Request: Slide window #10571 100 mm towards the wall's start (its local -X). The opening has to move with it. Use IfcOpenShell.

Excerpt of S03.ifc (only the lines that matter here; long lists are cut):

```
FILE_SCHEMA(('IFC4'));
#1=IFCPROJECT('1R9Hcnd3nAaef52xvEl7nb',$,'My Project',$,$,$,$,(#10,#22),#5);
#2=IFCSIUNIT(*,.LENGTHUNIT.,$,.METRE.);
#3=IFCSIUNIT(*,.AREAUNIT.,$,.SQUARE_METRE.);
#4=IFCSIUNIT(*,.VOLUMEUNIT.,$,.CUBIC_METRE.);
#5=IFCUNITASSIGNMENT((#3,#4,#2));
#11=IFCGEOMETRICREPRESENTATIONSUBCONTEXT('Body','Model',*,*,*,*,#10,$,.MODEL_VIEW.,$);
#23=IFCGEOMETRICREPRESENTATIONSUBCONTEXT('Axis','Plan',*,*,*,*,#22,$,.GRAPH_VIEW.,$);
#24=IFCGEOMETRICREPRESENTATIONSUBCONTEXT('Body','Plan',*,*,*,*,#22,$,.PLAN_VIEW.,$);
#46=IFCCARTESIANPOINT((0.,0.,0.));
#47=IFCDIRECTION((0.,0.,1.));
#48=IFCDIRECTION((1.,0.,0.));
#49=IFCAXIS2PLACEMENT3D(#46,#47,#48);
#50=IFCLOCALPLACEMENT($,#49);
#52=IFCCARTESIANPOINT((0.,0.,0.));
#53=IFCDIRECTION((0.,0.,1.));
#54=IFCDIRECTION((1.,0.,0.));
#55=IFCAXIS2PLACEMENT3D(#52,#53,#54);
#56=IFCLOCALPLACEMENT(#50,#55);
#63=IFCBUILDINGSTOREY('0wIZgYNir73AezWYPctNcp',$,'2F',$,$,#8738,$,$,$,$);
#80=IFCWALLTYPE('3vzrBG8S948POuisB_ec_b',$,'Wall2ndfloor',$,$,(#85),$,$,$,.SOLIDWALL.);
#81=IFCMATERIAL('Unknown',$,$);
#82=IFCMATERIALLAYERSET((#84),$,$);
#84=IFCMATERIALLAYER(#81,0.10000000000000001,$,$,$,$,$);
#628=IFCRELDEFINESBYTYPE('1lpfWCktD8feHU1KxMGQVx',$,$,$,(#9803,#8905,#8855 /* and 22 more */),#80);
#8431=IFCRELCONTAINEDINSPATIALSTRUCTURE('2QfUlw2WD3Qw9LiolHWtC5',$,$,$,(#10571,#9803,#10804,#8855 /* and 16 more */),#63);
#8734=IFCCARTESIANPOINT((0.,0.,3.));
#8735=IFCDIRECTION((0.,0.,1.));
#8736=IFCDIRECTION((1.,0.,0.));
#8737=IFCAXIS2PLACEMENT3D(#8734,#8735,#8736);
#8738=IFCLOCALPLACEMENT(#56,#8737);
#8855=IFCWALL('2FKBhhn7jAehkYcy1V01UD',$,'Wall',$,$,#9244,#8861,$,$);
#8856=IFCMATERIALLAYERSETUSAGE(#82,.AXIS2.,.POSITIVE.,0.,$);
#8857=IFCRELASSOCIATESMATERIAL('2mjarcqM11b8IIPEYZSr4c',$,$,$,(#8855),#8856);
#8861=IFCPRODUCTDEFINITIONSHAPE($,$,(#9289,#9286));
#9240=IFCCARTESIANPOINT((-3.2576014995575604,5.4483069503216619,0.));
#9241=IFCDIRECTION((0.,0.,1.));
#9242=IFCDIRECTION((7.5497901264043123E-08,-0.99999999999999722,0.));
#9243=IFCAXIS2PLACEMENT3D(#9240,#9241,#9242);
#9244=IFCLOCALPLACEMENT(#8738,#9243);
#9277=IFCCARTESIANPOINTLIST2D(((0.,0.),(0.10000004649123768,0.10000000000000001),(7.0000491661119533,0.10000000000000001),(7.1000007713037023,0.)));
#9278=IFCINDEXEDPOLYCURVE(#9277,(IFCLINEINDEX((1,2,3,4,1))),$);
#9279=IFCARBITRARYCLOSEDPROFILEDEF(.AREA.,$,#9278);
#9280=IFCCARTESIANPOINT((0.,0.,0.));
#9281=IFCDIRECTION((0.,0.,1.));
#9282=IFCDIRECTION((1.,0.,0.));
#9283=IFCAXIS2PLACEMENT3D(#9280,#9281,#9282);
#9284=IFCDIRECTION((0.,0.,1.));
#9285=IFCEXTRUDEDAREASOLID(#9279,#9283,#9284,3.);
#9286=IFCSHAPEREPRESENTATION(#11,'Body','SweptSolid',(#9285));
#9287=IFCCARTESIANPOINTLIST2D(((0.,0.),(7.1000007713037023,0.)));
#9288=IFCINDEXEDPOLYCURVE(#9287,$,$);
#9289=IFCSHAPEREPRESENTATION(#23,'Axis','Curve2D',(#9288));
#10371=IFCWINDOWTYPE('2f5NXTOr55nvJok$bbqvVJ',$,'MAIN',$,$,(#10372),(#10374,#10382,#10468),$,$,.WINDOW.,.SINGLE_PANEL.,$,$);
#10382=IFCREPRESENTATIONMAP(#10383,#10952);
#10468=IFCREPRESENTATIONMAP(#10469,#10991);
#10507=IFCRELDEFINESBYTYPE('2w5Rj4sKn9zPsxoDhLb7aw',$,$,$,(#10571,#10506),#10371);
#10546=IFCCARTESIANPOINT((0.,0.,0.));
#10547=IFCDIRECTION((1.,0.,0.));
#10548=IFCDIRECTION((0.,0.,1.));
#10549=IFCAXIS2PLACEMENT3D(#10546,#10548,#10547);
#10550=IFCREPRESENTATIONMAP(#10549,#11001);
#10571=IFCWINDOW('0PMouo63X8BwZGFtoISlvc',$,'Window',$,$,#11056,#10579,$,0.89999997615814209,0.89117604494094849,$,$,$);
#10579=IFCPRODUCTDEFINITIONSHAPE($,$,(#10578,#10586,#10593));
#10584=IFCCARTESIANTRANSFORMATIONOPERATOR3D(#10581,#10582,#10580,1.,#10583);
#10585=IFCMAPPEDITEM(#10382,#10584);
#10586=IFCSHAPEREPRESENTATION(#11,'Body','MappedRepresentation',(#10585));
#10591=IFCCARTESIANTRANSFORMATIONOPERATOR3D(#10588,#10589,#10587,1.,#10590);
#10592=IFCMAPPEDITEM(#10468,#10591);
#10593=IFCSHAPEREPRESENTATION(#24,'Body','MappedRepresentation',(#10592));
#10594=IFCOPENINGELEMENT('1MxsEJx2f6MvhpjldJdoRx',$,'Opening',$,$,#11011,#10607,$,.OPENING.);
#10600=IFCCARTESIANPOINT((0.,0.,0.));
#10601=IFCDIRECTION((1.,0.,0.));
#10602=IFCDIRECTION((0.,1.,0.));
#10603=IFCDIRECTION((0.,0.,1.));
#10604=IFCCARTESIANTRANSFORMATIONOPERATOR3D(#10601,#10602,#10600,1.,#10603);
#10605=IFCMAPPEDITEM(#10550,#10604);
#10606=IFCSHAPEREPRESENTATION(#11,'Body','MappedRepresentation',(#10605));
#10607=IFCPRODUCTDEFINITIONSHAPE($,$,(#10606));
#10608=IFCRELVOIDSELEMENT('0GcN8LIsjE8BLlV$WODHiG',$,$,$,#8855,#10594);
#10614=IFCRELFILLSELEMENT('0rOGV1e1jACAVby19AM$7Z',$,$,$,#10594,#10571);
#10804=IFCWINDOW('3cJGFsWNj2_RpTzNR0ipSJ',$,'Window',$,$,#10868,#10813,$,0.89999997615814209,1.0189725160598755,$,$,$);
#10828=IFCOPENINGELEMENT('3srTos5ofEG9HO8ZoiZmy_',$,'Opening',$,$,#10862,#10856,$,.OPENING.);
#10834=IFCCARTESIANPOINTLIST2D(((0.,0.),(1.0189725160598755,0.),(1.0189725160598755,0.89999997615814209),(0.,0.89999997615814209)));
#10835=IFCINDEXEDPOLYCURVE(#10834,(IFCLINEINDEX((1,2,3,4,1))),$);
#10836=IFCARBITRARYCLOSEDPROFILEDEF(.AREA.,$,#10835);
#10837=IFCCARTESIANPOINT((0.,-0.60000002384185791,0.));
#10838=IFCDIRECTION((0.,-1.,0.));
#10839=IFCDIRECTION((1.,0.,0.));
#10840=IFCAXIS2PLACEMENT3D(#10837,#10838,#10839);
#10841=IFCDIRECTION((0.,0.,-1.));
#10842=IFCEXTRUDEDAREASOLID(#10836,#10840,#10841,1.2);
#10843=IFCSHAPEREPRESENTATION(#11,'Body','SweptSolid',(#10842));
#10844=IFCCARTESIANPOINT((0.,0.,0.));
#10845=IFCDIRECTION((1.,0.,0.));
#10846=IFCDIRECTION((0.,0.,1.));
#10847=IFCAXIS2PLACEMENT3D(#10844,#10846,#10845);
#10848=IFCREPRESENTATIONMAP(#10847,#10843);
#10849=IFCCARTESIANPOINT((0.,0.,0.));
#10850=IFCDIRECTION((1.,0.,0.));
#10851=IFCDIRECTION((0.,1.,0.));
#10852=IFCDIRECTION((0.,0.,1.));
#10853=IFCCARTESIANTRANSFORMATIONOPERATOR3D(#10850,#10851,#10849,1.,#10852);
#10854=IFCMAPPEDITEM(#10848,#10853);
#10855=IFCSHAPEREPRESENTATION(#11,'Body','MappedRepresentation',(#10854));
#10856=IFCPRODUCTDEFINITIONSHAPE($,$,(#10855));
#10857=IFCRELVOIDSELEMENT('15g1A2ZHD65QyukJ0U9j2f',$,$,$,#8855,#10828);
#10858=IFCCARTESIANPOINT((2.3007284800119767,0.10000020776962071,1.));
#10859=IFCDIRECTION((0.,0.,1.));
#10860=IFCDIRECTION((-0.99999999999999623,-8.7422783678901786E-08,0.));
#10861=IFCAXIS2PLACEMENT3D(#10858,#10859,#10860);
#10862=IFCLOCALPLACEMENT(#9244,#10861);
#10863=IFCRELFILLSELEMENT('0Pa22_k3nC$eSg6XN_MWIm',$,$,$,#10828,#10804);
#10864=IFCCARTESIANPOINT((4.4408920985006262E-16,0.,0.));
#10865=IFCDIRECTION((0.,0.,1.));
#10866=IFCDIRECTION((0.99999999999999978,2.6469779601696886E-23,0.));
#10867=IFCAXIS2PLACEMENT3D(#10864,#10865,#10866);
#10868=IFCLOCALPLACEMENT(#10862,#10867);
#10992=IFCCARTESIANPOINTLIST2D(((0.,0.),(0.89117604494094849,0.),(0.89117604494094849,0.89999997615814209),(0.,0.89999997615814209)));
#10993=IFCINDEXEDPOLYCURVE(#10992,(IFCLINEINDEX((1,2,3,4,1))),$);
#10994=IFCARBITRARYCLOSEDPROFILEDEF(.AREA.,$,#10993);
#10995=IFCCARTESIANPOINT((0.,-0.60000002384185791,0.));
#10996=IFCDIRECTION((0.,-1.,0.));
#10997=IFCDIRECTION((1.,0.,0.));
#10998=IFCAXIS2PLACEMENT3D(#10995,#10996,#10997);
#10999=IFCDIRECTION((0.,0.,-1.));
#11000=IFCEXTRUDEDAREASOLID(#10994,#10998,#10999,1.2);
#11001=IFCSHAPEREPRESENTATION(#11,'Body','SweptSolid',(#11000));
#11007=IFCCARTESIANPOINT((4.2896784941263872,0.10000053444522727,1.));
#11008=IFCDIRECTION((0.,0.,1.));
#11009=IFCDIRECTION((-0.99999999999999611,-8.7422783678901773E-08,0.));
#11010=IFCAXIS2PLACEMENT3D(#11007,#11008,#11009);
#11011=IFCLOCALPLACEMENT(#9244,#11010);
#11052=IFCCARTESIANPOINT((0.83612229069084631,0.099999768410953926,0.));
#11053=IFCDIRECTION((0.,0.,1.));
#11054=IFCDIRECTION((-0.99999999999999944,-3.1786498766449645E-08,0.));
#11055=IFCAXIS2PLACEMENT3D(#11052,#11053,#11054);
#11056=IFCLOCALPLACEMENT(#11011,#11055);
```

```python
import ifcopenshell
import ifcopenshell.api.geometry
import ifcopenshell.util.placement

model = ifcopenshell.open("S03.ifc")

window = model.by_guid("0PMouo63X8BwZGFtoISlvc")
opening = window.FillsVoids[0].RelatingOpeningElement
wall = opening.VoidsElements[0].RelatingBuildingElement

wall_matrix = ifcopenshell.util.placement.get_local_placement(wall.ObjectPlacement)
shift = wall_matrix[:3, 0] * -0.1
before = ifcopenshell.util.placement.get_local_placement(window.ObjectPlacement)[:3, 3].copy()

# The window is placed relative to its opening, so it follows when the opening moves.
matrix = ifcopenshell.util.placement.get_local_placement(opening.ObjectPlacement)
matrix[:3, 3] += shift
ifcopenshell.api.geometry.edit_object_placement(
    model, product=opening, matrix=matrix, is_si=False, should_transform_children=True
)

after = ifcopenshell.util.placement.get_local_placement(window.ObjectPlacement)[:3, 3]
print("window moved by", (after - before).round(3) + 0.0)

model.write("S03_rev.ifc")
```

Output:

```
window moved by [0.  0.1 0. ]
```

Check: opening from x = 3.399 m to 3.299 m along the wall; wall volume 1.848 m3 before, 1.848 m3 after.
